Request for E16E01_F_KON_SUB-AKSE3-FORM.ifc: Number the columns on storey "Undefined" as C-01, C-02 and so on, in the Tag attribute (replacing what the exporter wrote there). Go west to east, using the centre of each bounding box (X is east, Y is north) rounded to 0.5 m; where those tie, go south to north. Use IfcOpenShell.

First a look at what the model holds.

```python
import ifcopenshell
import ifcopenshell.util.element
import ifcopenshell.util.placement

model = ifcopenshell.open("E16E01_F_KON_SUB-AKSE3-FORM.ifc")
print(model.schema)
storey = next(s for s in model.by_type("IfcBuildingStorey") if s.Name == "Undefined")
columns = [e for e in ifcopenshell.util.element.get_decomposition(storey) if e.is_a("IfcColumn")]
for e in sorted(columns, key=lambda e: e.id()):
    origin = ifcopenshell.util.placement.get_local_placement(e.ObjectPlacement)[:3, 3]
    print(e.id(), e.Tag, e.Name, origin.round(2) + 0.0, sep=" | ")
```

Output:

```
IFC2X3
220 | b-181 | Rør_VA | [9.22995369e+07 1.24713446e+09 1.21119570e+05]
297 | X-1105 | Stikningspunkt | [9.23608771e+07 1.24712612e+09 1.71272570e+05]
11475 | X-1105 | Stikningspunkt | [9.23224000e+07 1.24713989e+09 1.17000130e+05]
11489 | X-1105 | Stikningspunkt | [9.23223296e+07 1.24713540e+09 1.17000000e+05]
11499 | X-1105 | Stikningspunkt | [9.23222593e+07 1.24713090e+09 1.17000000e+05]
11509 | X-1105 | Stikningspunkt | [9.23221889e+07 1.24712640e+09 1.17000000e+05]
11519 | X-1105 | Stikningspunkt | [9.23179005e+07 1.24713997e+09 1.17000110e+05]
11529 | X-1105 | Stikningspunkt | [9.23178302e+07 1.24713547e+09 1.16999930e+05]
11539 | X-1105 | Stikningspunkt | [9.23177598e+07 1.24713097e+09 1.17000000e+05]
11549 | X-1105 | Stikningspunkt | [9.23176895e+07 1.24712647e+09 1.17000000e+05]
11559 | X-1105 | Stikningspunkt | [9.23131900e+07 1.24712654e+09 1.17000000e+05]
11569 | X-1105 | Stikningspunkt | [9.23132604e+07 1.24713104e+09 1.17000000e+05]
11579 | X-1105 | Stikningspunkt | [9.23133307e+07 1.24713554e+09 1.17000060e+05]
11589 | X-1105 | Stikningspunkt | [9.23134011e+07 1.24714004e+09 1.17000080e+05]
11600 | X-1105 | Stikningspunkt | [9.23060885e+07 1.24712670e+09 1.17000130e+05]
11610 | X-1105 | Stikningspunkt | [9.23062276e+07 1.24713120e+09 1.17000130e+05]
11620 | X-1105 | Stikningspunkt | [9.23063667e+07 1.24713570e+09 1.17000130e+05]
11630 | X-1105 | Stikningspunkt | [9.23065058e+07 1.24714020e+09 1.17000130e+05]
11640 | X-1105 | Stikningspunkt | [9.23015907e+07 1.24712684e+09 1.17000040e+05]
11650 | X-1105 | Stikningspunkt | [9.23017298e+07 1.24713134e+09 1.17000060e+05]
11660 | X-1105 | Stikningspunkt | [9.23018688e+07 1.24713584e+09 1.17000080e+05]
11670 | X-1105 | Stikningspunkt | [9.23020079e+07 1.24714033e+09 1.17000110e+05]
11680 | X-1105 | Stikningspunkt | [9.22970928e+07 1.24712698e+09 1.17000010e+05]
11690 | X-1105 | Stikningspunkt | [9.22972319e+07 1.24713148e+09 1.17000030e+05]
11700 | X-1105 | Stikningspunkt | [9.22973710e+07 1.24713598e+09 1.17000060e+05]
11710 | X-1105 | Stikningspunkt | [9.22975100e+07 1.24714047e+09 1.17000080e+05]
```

```python
import ifcopenshell
import ifcopenshell.geom
import ifcopenshell.util.element
import ifcopenshell.util.shape

model = ifcopenshell.open("E16E01_F_KON_SUB-AKSE3-FORM.ifc")
settings = ifcopenshell.geom.settings()
settings.set("use-world-coords", True)


def centre(element):
    shape = ifcopenshell.geom.create_shape(settings, element)
    return ifcopenshell.util.shape.get_bbox_centroid(shape.geometry)


storey = next(s for s in model.by_type("IfcBuildingStorey") if s.Name == "Undefined")
columns = [e for e in ifcopenshell.util.element.get_decomposition(storey) if e.is_a("IfcColumn")]

# Insertion points can sit at a corner or the storey origin, so sort by the geometry (in metres).
centres = {e: centre(e) for e in columns}
columns.sort(key=lambda e: (round(centres[e][0] / 0.5), centres[e][1]))

for i, e in enumerate(columns, start=1):
    number = f"C-{i:02d}"
    e.Tag = number
    print(e.id(), number)

model.write("E16E01_F_KON_SUB-AKSE3-FORM_v2.ifc")
```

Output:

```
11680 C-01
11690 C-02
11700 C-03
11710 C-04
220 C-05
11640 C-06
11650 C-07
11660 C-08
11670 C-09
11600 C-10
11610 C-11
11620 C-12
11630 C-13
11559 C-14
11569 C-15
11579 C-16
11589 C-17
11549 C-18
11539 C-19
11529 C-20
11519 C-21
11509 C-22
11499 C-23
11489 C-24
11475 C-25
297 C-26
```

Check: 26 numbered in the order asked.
